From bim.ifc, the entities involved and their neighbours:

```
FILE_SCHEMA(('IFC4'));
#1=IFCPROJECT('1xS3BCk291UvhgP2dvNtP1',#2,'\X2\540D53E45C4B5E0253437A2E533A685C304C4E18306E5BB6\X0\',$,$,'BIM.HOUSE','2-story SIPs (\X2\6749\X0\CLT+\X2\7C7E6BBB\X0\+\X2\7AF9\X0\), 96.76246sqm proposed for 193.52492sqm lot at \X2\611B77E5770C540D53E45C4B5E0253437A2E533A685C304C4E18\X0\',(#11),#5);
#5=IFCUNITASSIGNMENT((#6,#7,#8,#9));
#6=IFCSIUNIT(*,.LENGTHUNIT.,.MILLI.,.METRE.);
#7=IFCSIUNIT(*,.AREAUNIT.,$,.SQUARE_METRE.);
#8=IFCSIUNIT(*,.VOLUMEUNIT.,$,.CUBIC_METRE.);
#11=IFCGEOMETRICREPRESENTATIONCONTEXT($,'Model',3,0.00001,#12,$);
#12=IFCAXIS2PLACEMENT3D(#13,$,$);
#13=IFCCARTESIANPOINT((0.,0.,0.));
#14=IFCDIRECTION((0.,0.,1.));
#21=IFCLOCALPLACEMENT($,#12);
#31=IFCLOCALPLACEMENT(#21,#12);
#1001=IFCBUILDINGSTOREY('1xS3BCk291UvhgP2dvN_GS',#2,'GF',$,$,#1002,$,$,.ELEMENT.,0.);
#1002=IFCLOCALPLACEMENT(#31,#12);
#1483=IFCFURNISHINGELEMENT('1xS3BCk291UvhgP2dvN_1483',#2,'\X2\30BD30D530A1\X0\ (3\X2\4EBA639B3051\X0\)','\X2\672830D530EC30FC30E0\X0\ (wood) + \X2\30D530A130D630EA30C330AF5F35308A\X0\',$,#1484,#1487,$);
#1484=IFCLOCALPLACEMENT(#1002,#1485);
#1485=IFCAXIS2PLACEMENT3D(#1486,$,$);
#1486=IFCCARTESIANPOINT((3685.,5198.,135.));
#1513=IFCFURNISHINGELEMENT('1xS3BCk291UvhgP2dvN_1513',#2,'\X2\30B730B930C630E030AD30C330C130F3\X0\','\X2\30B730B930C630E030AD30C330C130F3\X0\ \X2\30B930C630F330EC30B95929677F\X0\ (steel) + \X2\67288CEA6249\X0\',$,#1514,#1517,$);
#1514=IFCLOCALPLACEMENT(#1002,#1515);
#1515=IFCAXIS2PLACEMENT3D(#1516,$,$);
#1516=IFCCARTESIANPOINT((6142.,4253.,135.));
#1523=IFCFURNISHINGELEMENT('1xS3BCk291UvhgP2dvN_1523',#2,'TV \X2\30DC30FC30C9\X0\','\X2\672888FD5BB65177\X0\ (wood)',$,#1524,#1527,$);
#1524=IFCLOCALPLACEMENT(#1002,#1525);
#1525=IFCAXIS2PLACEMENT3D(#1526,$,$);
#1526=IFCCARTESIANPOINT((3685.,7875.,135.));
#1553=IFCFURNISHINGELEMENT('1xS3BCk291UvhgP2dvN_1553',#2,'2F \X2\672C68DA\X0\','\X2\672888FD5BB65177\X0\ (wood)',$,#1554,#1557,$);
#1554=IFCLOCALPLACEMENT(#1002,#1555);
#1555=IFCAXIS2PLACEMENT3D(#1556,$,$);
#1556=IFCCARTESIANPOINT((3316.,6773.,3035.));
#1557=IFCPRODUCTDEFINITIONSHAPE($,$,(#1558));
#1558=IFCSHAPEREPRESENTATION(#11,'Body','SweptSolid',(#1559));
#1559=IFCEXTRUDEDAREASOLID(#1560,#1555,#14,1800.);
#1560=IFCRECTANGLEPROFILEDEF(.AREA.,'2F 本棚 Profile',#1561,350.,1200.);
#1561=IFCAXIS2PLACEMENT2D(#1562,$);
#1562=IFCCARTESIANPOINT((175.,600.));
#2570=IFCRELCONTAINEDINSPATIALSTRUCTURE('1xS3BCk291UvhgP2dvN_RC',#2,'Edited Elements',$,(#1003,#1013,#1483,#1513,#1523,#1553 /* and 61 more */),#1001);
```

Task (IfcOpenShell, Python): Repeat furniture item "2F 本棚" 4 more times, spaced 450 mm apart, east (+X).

```python
import numpy as np
import ifcopenshell
import ifcopenshell.api.geometry
import ifcopenshell.api.root
import ifcopenshell.util.element
import ifcopenshell.util.placement

model = ifcopenshell.open("bim.ifc")


def reuse_history(source, copy):
    """copy_class also copies each property set's owner history, people and application; keep the originals."""
    for rel in copy.IsDefinedBy:
        if rel.is_a("IfcRelDefinesByProperties") and (history := rel.RelatingPropertyDefinition.OwnerHistory):
            rel.RelatingPropertyDefinition.OwnerHistory = source.OwnerHistory
            ifcopenshell.util.element.remove_deep2(model, history)


source = model.by_guid("1xS3BCk291UvhgP2dvN_1553")
base = ifcopenshell.util.placement.get_local_placement(source.ObjectPlacement)
step = np.array([1.0, 0.0, 0.0]) * 450.0

for i in range(1, 5):
    copy = ifcopenshell.api.root.copy_class(model, product=source)
    copy.Representation = ifcopenshell.util.element.copy_deep(
        model, source.Representation, exclude=["IfcGeometricRepresentationContext", "IfcRepresentationMap"]
    )
    reuse_history(source, copy)
    matrix = base.copy()
    matrix[:3, 3] += i * step
    print("added at", matrix[:3, 3].round(3) + 0.0)
    ifcopenshell.api.geometry.edit_object_placement(model, product=copy, matrix=matrix, is_si=False)

model.write("bim_updated.ifc")
```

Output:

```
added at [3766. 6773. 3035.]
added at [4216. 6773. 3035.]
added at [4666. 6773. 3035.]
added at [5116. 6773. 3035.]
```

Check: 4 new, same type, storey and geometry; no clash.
